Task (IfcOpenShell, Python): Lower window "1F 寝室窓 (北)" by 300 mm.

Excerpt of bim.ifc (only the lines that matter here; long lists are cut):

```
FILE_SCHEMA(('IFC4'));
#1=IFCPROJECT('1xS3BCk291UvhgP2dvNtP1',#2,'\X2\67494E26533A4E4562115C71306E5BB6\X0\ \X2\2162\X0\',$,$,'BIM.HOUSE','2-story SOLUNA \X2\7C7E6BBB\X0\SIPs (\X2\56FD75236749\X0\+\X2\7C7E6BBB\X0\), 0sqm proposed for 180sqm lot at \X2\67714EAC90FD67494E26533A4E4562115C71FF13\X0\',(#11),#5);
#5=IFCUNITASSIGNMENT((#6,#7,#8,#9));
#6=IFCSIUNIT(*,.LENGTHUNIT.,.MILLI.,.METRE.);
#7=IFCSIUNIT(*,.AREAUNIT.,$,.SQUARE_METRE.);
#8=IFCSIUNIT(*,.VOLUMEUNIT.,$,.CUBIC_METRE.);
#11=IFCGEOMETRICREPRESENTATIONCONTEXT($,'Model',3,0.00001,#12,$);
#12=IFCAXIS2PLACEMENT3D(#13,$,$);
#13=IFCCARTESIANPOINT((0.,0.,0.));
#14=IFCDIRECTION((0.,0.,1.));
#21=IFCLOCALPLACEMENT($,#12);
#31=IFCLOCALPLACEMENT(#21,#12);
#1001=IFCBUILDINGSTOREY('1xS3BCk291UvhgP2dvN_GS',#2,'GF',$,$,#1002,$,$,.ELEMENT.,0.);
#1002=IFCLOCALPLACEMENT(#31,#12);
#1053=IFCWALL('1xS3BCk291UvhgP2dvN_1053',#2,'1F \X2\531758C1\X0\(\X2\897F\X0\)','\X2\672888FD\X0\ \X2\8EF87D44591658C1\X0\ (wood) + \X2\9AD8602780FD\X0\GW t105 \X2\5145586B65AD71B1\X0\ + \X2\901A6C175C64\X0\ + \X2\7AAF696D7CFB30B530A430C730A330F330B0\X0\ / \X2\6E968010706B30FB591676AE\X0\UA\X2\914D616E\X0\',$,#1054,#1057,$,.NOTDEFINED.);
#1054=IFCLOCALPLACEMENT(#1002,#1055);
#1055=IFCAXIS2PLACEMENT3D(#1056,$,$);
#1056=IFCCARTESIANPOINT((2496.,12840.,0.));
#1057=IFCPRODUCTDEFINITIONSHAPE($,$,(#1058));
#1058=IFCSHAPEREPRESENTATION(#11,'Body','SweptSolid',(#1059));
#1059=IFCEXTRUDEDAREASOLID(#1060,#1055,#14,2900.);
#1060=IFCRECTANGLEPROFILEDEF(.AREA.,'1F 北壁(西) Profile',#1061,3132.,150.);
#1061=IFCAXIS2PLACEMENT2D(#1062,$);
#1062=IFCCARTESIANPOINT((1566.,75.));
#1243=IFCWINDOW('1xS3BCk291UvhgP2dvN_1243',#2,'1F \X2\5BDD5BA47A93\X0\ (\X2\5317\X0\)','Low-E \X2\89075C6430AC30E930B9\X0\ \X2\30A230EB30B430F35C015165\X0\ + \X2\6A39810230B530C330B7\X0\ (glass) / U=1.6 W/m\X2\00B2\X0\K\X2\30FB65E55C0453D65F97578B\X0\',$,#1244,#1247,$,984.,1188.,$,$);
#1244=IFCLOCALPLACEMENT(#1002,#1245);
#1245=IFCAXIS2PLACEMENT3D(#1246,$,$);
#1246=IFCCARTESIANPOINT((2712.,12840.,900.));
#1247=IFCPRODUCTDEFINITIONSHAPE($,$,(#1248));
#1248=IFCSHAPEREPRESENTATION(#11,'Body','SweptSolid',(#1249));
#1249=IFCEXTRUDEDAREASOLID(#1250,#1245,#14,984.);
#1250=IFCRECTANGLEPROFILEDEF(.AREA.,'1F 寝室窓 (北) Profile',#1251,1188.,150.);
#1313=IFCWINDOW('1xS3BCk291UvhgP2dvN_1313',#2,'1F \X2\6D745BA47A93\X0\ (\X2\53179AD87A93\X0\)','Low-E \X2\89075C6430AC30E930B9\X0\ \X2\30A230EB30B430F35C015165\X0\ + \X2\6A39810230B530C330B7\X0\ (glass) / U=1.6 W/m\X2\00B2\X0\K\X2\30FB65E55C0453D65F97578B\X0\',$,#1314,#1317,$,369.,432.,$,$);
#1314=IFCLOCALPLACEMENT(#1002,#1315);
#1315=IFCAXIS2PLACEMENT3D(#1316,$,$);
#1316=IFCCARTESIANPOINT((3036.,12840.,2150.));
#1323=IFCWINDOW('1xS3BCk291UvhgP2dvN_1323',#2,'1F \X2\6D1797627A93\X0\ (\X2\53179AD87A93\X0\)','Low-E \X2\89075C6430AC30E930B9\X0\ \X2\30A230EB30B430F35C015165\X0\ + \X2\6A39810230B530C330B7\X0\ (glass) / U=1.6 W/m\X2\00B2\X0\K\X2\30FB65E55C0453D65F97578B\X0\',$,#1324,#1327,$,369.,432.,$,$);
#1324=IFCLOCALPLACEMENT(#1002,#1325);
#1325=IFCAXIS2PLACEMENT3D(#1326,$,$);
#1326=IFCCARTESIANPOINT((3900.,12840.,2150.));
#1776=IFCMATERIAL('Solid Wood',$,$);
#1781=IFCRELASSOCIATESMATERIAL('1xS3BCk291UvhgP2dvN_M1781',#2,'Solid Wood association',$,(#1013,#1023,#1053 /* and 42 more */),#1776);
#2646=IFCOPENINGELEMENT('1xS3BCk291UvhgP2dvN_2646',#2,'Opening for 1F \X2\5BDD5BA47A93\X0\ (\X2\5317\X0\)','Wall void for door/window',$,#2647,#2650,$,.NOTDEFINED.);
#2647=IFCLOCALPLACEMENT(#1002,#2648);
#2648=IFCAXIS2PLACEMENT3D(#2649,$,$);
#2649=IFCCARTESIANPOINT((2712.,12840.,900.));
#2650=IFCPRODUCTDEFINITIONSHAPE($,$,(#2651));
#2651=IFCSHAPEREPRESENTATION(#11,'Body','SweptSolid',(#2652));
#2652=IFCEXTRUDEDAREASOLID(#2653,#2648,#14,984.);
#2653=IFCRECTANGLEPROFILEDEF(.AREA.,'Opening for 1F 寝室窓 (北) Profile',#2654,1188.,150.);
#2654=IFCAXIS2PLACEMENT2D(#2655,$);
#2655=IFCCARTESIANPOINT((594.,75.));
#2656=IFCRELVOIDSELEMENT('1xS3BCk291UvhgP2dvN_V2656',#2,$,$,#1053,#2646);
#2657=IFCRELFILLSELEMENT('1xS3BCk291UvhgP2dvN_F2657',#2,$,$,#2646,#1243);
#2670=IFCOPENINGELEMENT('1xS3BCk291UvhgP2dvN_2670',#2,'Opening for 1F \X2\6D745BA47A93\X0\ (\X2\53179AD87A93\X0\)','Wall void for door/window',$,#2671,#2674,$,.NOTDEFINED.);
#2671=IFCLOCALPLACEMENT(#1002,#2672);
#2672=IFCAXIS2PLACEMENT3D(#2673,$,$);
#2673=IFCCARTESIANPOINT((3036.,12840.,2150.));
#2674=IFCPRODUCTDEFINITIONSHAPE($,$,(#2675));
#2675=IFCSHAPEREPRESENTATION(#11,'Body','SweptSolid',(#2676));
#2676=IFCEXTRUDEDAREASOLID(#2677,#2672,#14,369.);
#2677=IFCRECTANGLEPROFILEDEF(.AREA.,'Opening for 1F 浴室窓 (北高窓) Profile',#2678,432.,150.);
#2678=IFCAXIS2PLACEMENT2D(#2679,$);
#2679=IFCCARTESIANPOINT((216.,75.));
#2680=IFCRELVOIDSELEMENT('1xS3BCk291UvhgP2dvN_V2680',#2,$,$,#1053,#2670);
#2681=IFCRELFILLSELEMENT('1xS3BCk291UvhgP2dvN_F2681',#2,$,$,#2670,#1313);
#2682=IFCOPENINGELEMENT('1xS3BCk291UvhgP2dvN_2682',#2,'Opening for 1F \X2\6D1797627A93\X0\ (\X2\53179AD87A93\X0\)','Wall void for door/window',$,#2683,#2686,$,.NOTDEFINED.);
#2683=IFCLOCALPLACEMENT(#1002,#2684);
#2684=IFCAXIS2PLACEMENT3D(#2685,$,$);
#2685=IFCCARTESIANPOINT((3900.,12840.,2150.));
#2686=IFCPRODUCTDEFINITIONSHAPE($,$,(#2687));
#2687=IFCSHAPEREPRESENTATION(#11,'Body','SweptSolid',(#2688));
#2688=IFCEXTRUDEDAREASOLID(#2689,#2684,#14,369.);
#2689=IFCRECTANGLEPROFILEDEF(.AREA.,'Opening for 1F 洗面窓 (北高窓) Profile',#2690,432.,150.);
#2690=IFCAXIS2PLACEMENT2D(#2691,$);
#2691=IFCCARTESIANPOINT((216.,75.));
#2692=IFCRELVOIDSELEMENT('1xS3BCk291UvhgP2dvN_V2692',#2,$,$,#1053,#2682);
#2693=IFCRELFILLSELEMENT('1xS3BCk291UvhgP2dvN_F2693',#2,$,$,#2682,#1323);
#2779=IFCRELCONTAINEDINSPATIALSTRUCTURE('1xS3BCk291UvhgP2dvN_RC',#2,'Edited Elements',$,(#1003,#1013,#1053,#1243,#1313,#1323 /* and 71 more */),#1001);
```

```python
import numpy as np
import ifcopenshell
import ifcopenshell.api.geometry
import ifcopenshell.util.placement
import ifcopenshell.util.unit

model = ifcopenshell.open("bim.ifc")
unit_scale = ifcopenshell.util.unit.calculate_unit_scale(model)

window = model.by_guid("1xS3BCk291UvhgP2dvN_1243")
opening = window.FillsVoids[0].RelatingOpeningElement
dz = -300.0

shift = np.array([0.0, 0.0, dz])
# The window is not placed relative to its opening, so move both.
for product in (opening, window):
    matrix = ifcopenshell.util.placement.get_local_placement(product.ObjectPlacement)
    matrix[:3, 3] += shift
    ifcopenshell.api.geometry.edit_object_placement(model, product=product, matrix=matrix, is_si=False)

print(f"moved by {dz * unit_scale:+.3f} m")

model.write("bim_edited.ifc")
```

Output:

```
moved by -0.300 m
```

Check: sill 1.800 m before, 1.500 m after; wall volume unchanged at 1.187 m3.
